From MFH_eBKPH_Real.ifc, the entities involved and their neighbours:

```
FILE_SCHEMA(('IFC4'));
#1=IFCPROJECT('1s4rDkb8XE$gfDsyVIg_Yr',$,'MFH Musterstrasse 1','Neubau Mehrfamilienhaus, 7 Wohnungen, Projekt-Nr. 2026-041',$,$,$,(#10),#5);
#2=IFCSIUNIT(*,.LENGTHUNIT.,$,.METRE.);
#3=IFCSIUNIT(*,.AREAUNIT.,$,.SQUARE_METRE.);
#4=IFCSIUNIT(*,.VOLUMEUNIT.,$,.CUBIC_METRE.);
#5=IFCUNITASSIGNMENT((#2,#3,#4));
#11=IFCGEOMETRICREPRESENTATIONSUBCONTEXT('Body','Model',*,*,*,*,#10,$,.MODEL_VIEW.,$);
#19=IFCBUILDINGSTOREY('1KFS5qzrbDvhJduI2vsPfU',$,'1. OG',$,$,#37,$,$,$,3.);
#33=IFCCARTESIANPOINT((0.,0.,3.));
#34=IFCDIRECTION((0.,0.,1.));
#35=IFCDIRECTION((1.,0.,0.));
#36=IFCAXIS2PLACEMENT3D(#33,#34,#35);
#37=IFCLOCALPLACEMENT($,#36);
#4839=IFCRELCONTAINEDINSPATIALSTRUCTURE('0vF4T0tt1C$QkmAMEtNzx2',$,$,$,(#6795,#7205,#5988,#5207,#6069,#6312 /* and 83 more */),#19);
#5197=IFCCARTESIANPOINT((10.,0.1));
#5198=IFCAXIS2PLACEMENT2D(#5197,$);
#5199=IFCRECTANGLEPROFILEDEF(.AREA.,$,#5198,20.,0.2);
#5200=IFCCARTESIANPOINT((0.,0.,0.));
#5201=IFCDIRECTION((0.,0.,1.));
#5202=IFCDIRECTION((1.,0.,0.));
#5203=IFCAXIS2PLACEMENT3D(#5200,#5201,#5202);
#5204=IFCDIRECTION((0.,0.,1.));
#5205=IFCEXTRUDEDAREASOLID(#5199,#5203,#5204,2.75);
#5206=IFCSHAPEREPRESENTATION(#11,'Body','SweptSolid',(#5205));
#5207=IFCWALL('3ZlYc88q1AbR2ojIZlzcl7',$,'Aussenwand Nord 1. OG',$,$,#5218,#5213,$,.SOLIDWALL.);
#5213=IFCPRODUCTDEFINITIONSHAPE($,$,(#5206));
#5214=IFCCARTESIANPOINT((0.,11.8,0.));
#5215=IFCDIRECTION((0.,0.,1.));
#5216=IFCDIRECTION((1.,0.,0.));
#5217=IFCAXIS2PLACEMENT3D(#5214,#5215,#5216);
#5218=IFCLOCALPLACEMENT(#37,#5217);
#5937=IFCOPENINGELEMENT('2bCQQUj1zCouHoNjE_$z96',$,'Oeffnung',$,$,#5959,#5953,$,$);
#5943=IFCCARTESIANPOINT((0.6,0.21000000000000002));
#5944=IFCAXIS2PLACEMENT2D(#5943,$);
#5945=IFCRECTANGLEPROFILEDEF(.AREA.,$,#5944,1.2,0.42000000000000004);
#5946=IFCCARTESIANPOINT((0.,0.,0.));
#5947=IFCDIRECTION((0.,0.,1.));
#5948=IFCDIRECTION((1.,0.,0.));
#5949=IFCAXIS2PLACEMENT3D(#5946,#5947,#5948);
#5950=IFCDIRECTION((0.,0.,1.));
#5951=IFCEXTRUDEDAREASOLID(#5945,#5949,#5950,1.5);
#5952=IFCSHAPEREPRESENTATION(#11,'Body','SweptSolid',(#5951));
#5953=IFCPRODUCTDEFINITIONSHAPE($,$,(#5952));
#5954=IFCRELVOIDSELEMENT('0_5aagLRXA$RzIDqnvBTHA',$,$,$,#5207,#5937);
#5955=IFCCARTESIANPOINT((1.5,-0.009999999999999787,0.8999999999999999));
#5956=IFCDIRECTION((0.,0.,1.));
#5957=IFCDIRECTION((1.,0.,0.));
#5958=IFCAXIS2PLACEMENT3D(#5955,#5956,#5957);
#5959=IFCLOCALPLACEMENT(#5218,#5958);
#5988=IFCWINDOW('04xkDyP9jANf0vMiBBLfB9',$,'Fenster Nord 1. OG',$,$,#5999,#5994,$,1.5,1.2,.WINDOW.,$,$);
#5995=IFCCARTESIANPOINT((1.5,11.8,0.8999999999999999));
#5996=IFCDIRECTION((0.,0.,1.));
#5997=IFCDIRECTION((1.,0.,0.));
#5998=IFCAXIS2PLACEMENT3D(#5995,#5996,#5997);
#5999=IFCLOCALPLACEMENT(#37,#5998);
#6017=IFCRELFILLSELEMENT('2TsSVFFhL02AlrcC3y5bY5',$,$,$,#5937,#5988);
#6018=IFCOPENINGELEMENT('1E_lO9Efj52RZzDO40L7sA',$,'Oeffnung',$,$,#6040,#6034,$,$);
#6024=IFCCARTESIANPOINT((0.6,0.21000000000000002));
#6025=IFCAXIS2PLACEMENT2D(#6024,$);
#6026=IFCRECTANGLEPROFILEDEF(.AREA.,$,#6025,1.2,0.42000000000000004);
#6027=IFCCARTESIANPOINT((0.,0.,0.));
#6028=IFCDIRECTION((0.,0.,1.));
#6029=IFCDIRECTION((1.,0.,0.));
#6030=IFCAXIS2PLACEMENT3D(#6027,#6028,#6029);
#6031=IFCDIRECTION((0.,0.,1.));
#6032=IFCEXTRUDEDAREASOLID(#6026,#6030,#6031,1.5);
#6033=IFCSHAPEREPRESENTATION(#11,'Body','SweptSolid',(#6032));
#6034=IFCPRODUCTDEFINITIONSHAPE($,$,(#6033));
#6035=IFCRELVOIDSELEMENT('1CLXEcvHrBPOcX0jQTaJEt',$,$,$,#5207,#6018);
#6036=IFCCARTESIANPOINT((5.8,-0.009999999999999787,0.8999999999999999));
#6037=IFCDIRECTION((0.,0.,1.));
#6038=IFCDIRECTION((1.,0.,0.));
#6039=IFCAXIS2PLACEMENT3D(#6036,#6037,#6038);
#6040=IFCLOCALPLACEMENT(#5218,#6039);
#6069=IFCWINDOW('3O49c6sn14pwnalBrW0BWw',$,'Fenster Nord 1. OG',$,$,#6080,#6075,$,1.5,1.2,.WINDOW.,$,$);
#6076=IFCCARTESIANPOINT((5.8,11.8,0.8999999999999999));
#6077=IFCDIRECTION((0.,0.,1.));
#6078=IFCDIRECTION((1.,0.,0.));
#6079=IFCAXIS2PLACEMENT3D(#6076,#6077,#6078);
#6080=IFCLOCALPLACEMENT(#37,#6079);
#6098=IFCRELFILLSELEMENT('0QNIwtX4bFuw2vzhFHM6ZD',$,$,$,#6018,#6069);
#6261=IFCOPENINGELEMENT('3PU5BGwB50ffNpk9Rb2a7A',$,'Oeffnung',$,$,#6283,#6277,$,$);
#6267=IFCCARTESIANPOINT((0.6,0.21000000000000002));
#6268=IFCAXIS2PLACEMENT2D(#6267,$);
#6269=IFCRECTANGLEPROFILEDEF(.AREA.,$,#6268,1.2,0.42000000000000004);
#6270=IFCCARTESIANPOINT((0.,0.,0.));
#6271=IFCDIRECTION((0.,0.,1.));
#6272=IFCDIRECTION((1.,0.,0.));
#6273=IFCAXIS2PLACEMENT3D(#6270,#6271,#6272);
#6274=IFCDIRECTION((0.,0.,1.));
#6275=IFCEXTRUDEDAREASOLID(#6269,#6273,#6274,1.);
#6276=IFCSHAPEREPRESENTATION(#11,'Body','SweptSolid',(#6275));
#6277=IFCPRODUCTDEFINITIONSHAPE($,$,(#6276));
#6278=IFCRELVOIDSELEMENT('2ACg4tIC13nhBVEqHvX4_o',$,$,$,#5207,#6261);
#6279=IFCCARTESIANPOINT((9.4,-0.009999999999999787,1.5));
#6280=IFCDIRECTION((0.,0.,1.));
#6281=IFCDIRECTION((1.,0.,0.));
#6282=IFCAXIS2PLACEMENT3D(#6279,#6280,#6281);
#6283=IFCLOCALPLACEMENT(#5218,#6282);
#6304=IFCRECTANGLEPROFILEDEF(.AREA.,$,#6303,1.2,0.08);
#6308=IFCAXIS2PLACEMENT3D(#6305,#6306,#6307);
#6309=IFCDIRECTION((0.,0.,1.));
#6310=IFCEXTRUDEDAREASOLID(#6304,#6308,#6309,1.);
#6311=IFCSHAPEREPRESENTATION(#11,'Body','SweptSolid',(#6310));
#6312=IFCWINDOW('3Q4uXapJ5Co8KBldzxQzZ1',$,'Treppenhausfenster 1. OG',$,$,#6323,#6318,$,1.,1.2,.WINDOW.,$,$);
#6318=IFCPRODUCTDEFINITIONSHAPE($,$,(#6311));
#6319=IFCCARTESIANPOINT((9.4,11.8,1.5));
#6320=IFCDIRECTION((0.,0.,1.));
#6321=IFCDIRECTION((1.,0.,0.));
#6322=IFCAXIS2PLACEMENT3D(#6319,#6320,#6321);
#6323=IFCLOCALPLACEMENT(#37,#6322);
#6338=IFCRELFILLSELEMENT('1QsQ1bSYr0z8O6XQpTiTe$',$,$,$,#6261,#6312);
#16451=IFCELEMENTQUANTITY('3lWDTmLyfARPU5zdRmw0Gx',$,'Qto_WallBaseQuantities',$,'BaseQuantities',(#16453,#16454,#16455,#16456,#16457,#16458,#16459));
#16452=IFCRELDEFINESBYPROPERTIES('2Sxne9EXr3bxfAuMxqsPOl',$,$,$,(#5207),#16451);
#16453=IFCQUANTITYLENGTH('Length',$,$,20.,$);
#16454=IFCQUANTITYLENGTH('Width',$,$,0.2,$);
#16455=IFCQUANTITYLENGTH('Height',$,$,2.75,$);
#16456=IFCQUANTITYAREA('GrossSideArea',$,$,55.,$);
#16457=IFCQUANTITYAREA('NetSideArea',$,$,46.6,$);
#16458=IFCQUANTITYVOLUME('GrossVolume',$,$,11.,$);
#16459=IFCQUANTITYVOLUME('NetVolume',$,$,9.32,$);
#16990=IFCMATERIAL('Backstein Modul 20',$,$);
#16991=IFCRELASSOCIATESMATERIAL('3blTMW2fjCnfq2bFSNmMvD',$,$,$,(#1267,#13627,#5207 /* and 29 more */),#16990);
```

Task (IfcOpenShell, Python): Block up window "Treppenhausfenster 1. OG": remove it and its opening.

```python
import ifcopenshell
import ifcopenshell.api.feature
import ifcopenshell.api.pset
import ifcopenshell.api.root
import ifcopenshell.geom
import ifcopenshell.util.element
import ifcopenshell.util.shape
import ifcopenshell.util.unit

model = ifcopenshell.open("MFH_eBKPH_Real.ifc")
area_scale = ifcopenshell.util.unit.calculate_unit_scale(model, "AREAUNIT")
volume_scale = ifcopenshell.util.unit.calculate_unit_scale(model, "VOLUMEUNIT")
settings = ifcopenshell.geom.settings()


def volume(element):
    """Net volume in cubic metres, openings subtracted."""
    shape = ifcopenshell.geom.create_shape(settings, element)
    return ifcopenshell.util.shape.get_volume(shape.geometry)


window = model.by_guid("3Q4uXapJ5Co8KBldzxQzZ1")
opening = window.FillsVoids[0].RelatingOpeningElement
wall = opening.VoidsElements[0].RelatingBuildingElement
before = volume(wall)

ifcopenshell.api.root.remove_product(model, product=window)
ifcopenshell.api.feature.remove_feature(model, feature=opening)

after = volume(wall)
thickness = 0.2  # wall thickness in metres

# Update the wall's stored quantities.
qto = model.by_id(ifcopenshell.util.element.get_pset(wall, "Qto_WallBaseQuantities", should_inherit=False)["id"])
ifcopenshell.api.pset.edit_qto(model, qto=qto, properties={
    "NetSideArea": after / thickness / area_scale,
    "NetVolume": after / volume_scale,
})

print(f"wall volume {before:.3f} -> {after:.3f} m3")

model.write("MFH_eBKPH_Real_edited.ifc")
```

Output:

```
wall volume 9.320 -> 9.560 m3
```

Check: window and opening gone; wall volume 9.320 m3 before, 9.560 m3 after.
